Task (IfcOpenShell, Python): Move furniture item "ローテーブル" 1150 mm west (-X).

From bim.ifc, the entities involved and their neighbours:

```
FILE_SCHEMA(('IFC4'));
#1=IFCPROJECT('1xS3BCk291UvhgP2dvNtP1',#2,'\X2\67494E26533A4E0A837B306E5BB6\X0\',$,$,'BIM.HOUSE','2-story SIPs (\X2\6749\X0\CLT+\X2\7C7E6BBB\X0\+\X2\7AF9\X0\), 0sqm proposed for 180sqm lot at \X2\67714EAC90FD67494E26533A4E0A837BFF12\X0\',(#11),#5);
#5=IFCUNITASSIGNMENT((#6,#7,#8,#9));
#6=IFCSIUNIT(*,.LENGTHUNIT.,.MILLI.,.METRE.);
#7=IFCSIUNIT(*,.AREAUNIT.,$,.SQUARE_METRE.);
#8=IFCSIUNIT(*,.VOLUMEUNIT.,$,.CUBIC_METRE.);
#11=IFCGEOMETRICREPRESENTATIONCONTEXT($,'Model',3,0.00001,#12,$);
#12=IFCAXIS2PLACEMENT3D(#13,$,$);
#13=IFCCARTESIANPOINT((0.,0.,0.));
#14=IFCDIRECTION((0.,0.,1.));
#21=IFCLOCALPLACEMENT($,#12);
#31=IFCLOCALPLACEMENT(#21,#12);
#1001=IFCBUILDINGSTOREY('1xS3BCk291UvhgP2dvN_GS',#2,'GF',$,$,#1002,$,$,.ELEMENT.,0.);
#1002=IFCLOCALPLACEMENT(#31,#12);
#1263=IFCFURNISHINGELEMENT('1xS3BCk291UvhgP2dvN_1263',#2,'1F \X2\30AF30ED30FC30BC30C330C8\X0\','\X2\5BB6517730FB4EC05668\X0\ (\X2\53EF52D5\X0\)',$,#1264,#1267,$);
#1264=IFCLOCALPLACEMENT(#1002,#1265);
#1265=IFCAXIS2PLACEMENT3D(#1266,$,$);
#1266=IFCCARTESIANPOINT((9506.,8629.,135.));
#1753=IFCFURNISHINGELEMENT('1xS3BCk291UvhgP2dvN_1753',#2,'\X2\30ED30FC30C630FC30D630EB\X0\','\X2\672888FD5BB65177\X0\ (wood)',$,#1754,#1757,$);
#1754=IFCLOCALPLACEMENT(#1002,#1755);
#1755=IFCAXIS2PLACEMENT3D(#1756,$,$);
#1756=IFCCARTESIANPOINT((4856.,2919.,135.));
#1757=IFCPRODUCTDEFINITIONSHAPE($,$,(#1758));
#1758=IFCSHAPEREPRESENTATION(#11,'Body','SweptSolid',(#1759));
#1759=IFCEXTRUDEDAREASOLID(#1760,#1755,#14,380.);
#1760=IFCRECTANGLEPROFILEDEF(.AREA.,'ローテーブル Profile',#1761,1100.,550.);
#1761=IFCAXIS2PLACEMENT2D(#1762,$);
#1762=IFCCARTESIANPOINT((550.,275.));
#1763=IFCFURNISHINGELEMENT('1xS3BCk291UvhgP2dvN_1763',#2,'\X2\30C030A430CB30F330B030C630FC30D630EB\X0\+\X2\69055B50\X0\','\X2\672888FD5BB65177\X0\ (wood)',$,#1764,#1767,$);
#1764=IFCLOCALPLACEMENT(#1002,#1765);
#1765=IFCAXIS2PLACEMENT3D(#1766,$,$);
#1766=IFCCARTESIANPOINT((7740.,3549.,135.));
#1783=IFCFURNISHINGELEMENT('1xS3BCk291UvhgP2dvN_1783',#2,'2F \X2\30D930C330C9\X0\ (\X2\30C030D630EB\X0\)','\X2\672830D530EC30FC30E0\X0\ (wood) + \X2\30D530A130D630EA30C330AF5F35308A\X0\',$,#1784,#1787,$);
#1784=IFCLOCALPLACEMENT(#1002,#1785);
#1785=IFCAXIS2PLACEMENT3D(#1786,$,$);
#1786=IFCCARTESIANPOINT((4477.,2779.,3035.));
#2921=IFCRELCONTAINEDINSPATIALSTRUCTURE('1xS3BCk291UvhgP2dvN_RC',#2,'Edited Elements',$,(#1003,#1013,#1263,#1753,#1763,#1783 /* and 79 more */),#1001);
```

```python
import ifcopenshell
import ifcopenshell.api.geometry
import ifcopenshell.util.placement

model = ifcopenshell.open("bim.ifc")

item = model.by_guid("1xS3BCk291UvhgP2dvN_1753")
matrix = ifcopenshell.util.placement.get_local_placement(item.ObjectPlacement)
matrix[0, 3] -= 1150.0
ifcopenshell.api.geometry.edit_object_placement(model, product=item, matrix=matrix, is_si=False)

print(ifcopenshell.util.placement.get_local_placement(item.ObjectPlacement).round(3) + 0.0)

model.write("bim_rev.ifc")
```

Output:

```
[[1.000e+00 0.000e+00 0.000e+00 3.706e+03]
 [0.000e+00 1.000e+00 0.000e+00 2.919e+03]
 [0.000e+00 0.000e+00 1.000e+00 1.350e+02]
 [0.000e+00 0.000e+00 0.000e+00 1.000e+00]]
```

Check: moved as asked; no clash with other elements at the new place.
